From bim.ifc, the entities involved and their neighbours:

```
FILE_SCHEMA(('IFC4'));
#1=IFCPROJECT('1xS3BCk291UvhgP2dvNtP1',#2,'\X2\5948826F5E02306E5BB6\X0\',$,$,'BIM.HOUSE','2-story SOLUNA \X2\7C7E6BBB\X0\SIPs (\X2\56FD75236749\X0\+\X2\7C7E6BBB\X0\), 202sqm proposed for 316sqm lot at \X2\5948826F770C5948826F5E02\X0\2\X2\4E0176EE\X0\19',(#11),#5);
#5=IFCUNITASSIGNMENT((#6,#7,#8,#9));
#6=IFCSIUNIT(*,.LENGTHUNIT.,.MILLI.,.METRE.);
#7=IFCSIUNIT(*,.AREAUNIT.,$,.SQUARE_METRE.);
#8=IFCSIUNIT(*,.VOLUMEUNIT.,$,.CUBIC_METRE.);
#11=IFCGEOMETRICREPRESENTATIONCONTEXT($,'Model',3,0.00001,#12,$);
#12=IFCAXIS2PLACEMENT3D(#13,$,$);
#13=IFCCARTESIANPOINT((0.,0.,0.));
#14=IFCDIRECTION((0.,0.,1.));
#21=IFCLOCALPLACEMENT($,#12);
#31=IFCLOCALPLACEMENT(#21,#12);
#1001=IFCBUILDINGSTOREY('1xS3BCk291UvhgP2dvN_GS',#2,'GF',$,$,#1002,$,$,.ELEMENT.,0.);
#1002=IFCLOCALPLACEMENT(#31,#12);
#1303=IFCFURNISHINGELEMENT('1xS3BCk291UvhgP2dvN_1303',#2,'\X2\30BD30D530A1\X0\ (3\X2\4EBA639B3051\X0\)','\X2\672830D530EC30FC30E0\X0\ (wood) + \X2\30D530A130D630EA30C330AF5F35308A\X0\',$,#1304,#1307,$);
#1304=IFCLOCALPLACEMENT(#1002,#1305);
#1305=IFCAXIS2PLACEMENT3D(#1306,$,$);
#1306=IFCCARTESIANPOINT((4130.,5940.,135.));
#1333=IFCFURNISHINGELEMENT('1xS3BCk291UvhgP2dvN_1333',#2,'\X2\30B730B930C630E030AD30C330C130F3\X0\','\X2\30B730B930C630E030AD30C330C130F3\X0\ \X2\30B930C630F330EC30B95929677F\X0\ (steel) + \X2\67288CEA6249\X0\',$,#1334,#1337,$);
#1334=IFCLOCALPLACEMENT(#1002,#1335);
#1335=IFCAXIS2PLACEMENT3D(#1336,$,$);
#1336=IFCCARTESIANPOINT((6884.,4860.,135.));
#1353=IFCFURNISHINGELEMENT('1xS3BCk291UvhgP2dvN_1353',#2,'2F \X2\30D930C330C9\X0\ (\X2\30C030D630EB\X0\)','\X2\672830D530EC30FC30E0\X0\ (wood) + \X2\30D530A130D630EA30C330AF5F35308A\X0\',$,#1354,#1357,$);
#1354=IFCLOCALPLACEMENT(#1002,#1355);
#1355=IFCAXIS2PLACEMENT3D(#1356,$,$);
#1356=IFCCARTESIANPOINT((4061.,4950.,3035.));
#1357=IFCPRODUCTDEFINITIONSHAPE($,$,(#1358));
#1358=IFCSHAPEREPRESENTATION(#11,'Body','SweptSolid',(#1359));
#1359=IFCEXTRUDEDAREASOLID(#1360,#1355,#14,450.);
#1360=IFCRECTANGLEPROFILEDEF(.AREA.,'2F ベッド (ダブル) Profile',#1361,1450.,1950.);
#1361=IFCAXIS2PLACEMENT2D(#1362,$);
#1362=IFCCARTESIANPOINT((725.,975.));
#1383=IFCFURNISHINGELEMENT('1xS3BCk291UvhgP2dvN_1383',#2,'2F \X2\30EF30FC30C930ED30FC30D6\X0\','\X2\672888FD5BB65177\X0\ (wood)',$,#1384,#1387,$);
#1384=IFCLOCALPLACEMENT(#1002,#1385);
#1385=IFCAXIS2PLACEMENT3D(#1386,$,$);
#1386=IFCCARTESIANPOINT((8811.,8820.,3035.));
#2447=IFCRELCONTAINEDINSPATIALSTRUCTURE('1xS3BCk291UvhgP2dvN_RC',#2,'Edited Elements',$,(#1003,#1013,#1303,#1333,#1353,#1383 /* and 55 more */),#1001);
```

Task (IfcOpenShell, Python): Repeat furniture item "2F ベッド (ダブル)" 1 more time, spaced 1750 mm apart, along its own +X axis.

```python
import ifcopenshell
import ifcopenshell.api.geometry
import ifcopenshell.api.root
import ifcopenshell.util.element
import ifcopenshell.util.placement
import ifcopenshell.util.unit

model = ifcopenshell.open("bim.ifc")
unit_scale = ifcopenshell.util.unit.calculate_unit_scale(model)


def reuse_history(source, copy):
    """copy_class also copies each property set's owner history, people and application; keep the originals."""
    for rel in copy.IsDefinedBy:
        if rel.is_a("IfcRelDefinesByProperties") and (history := rel.RelatingPropertyDefinition.OwnerHistory):
            rel.RelatingPropertyDefinition.OwnerHistory = source.OwnerHistory
            ifcopenshell.util.element.remove_deep2(model, history)


source = model.by_guid("1xS3BCk291UvhgP2dvN_1353")
base = ifcopenshell.util.placement.get_local_placement(source.ObjectPlacement)
step = base[:3, 0] * 1.75 / unit_scale

for i in range(1, 2):
    copy = ifcopenshell.api.root.copy_class(model, product=source)
    copy.Representation = ifcopenshell.util.element.copy_deep(
        model, source.Representation, exclude=["IfcGeometricRepresentationContext", "IfcRepresentationMap"]
    )
    reuse_history(source, copy)
    matrix = base.copy()
    matrix[:3, 3] += i * step
    print("added at", matrix[:3, 3].round(3) + 0.0)
    ifcopenshell.api.geometry.edit_object_placement(model, product=copy, matrix=matrix, is_si=False)

model.write("bim_edited.ifc")
```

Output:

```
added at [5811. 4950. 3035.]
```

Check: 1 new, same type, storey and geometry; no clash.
